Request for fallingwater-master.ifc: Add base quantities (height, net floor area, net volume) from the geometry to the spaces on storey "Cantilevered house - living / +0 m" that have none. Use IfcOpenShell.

First a look at what the model holds.

```python
import ifcopenshell
import ifcopenshell.util.element
import ifcopenshell.util.unit

model = ifcopenshell.open("fallingwater-master.ifc")
print(model.schema)
for unit_type in ("LENGTHUNIT", "AREAUNIT", "VOLUMEUNIT"):
    print(unit_type, ifcopenshell.util.unit.calculate_unit_scale(model, unit_type))
storey = next(s for s in model.by_type("IfcBuildingStorey") if s.Name == "Cantilevered house - living / +0 m")
spaces = [e for e in ifcopenshell.util.element.get_decomposition(storey) if e.is_a("IfcSpace")]
for e in sorted(spaces, key=lambda e: e.id()):
    print(e.id(), e.is_a(), e.Name, list(ifcopenshell.util.element.get_psets(e, qtos_only=True)), sep=" | ")
```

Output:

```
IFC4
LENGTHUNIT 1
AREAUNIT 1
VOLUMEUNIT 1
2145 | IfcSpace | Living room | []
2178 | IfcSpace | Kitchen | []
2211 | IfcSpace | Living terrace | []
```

```python
import ifcopenshell
import ifcopenshell.api.pset
import ifcopenshell.geom
import ifcopenshell.util.element
import ifcopenshell.util.shape
import ifcopenshell.util.unit

model = ifcopenshell.open("fallingwater-master.ifc")
unit_scale = ifcopenshell.util.unit.calculate_unit_scale(model)
area_scale = ifcopenshell.util.unit.calculate_unit_scale(model, "AREAUNIT")
volume_scale = ifcopenshell.util.unit.calculate_unit_scale(model, "VOLUMEUNIT")
settings = ifcopenshell.geom.settings()

storey = next(s for s in model.by_type("IfcBuildingStorey") if s.Name == "Cantilevered house - living / +0 m")
spaces = [e for e in ifcopenshell.util.element.get_decomposition(storey) if e.is_a("IfcSpace")]

for e in sorted(spaces, key=lambda e: e.id()):
    if ifcopenshell.util.element.get_psets(e, qtos_only=True, should_inherit=False):
        continue
    # Geometry comes back in metres, in the element's own axes.
    shape = ifcopenshell.geom.create_shape(settings, e)
    values = {
        "Height": ifcopenshell.util.shape.get_z(shape.geometry) / unit_scale,
        "NetFloorArea": ifcopenshell.util.shape.get_footprint_area(shape.geometry) / area_scale,
        "NetVolume": ifcopenshell.util.shape.get_volume(shape.geometry) / volume_scale,
    }
    qto = ifcopenshell.api.pset.add_qto(model, product=e, name="Qto_SpaceBaseQuantities")
    ifcopenshell.api.pset.edit_qto(model, qto=qto, properties=values)
    print(e.id(), {k: round(v, 3) for k, v in values.items()})

model.write("fallingwater-master_updated.ifc")
```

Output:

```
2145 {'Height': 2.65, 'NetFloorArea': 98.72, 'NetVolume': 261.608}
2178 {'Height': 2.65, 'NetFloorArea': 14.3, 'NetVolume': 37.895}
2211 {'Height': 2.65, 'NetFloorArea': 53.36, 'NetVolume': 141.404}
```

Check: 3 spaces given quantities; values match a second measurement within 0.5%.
